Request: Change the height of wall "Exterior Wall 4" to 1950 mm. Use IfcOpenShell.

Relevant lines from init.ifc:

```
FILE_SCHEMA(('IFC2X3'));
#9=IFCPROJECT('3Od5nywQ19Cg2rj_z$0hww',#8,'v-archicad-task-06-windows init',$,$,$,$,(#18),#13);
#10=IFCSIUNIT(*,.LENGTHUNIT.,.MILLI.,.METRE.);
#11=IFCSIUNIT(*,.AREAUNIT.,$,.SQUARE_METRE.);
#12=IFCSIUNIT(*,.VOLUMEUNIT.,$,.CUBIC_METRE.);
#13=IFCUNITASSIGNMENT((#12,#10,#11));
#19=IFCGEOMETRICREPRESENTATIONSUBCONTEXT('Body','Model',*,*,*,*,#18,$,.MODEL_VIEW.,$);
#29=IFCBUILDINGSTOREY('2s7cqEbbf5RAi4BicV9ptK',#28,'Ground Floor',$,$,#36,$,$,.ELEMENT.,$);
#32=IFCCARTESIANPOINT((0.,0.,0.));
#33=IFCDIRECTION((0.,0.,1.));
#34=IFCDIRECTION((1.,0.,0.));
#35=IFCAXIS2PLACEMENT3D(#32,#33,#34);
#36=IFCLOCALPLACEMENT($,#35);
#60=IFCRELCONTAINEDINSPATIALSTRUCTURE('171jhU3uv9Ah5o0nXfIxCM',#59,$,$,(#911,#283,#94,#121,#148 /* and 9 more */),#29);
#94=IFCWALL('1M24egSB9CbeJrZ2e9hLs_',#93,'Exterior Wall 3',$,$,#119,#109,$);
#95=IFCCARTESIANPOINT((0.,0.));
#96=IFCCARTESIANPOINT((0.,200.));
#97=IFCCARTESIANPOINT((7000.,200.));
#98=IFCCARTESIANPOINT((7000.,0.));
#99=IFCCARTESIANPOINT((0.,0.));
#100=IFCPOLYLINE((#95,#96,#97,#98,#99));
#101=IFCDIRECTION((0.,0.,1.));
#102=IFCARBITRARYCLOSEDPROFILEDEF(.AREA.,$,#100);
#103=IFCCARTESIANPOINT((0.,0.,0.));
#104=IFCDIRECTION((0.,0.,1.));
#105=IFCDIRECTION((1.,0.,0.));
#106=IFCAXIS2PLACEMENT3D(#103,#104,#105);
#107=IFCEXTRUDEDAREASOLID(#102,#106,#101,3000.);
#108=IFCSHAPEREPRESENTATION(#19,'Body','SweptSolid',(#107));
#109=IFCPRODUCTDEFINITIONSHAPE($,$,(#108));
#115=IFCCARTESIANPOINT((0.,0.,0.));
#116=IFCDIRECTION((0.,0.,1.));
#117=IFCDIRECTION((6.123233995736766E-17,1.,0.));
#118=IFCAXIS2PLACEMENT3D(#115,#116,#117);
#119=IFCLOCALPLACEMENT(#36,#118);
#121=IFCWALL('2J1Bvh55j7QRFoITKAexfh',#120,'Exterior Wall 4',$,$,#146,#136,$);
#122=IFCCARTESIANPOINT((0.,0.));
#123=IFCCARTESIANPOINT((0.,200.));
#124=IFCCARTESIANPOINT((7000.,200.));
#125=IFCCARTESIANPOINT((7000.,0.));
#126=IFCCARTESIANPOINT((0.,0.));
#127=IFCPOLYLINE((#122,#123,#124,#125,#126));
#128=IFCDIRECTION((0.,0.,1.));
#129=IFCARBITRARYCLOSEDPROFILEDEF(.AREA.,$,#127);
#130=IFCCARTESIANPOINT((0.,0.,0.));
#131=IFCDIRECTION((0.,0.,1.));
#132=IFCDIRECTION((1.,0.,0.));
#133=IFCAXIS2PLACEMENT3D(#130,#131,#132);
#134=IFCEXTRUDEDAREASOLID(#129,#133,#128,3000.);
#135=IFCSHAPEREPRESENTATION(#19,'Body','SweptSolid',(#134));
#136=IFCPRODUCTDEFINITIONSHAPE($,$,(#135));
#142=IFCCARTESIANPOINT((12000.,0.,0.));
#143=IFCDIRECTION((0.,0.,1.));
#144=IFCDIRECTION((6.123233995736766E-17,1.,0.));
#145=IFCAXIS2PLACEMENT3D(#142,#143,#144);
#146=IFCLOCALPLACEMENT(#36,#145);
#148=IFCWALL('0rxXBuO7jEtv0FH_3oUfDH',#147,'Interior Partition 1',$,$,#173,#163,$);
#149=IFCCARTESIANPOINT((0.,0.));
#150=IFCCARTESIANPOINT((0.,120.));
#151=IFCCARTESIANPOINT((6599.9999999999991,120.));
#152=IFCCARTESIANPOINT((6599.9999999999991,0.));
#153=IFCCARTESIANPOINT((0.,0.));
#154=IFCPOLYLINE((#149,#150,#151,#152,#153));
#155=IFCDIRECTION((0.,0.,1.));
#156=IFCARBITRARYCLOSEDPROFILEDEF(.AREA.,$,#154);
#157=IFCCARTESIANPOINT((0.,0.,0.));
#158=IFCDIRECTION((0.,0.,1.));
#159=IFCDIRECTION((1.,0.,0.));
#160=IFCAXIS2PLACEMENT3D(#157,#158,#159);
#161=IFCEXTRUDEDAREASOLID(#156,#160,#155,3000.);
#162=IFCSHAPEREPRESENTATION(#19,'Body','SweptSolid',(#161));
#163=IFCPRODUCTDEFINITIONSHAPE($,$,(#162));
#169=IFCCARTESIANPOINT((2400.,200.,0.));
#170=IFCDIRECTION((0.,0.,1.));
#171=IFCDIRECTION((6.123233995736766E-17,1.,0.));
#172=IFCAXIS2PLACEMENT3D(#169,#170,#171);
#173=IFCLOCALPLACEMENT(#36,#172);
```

```python
import ifcopenshell
import ifcopenshell.geom
import ifcopenshell.util.representation
import ifcopenshell.util.shape

model = ifcopenshell.open("init.ifc")
settings = ifcopenshell.geom.settings()


def volume(element):
    """Net volume in cubic metres, openings subtracted."""
    shape = ifcopenshell.geom.create_shape(settings, element)
    return ifcopenshell.util.shape.get_volume(shape.geometry)


wall = model.by_guid("2J1Bvh55j7QRFoITKAexfh")
before = volume(wall)

body = ifcopenshell.util.representation.get_representation(wall, "Model", "Body")
solid = body.Items[0]
old_height = solid.Depth
solid.Depth = 1950.0
after = volume(wall)

print(f"height {old_height:g} -> {solid.Depth:g}, volume {before:.3f} -> {after:.3f} m3")

model.write("init_v2.ifc")
```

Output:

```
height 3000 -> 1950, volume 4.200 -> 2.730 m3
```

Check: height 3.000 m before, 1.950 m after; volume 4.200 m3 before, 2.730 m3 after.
